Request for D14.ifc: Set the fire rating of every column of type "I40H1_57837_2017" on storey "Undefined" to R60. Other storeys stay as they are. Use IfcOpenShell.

First a look at what the model holds.

```python
import ifcopenshell
import ifcopenshell.util.element

model = ifcopenshell.open("D14.ifc")
print(model.schema)
storey = next(s for s in model.by_type("IfcBuildingStorey") if s.Name == "Undefined")
columns = [e for e in ifcopenshell.util.element.get_decomposition(storey) if e.is_a("IfcColumn")]
seen = {}
for e in columns:
    element_type = ifcopenshell.util.element.get_type(e)
    key = (element_type.Name if element_type != e and element_type else None, ifcopenshell.util.element.get_pset(e, "Pset_ColumnCommon", "FireRating"))
    seen[key] = seen.get(key, 0) + 1
for (name, value), count in sorted(seen.items(), key=str):
    print(count, "x", name, "|", value)
```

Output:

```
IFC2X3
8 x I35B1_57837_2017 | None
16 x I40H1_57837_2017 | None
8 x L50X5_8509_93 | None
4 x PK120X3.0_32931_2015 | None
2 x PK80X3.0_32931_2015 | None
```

```python
import ifcopenshell
import ifcopenshell.api.pset
import ifcopenshell.util.element

model = ifcopenshell.open("D14.ifc")

storey = next(s for s in model.by_type("IfcBuildingStorey") if s.Name == "Undefined")
columns = [e for e in ifcopenshell.util.element.get_decomposition(storey) if e.is_a("IfcColumn")]

count = 0
for e in columns:
    element_type = ifcopenshell.util.element.get_type(e)
    if element_type in (None, e) or element_type.Name != "I40H1_57837_2017":
        continue
    found = ifcopenshell.util.element.get_pset(e, "Pset_ColumnCommon", should_inherit=False)
    if found:
        pset = model.by_id(found["id"])
        if len(ifcopenshell.util.element.get_elements_by_pset(pset)) > 1:
            pset = ifcopenshell.api.pset.unshare_pset(model, products=[e], pset=pset)[0]
    else:
        pset = ifcopenshell.api.pset.add_pset(model, product=e, name="Pset_ColumnCommon")
    ifcopenshell.api.pset.edit_pset(model, pset=pset, properties={"FireRating": "R60"})
    count += 1

print(count, "columns updated")

model.write("D14_edited.ifc")
```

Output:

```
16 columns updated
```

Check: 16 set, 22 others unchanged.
